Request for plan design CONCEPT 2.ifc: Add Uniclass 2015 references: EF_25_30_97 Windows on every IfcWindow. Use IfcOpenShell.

First a look at what the model holds.

```python
import ifcopenshell

model = ifcopenshell.open("plan design CONCEPT 2.ifc")
print(model.schema)
print("classifications:", [c.Name for c in model.by_type("IfcClassification")])
for ifc_class in ("IfcDoor", "IfcRoof", "IfcStair", "IfcWall", "IfcWindow"):
    print(ifc_class, len(model.by_type(ifc_class)))
```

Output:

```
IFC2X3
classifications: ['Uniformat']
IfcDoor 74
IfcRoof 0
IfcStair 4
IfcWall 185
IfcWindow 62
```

```python
import ifcopenshell
import ifcopenshell.api.classification

model = ifcopenshell.open("plan design CONCEPT 2.ifc")

# IFC2X3 requires Source and Edition and has no link from the project to the system.
system = model.create_entity("IfcClassification", Source="NBS", Edition="2015", Name="Uniclass 2015")

codes = {
    "IfcWindow": ("EF_25_30_97", "Windows"),
}
for ifc_class, (code, name) in codes.items():
    products = model.by_type(ifc_class)
    ifcopenshell.api.classification.add_reference(
        model, products=products, classification=system, identification=code, name=name
    )
    print(code, len(products))

model.write("plan design CONCEPT 2_rev.ifc")
```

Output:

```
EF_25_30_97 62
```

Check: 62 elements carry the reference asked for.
